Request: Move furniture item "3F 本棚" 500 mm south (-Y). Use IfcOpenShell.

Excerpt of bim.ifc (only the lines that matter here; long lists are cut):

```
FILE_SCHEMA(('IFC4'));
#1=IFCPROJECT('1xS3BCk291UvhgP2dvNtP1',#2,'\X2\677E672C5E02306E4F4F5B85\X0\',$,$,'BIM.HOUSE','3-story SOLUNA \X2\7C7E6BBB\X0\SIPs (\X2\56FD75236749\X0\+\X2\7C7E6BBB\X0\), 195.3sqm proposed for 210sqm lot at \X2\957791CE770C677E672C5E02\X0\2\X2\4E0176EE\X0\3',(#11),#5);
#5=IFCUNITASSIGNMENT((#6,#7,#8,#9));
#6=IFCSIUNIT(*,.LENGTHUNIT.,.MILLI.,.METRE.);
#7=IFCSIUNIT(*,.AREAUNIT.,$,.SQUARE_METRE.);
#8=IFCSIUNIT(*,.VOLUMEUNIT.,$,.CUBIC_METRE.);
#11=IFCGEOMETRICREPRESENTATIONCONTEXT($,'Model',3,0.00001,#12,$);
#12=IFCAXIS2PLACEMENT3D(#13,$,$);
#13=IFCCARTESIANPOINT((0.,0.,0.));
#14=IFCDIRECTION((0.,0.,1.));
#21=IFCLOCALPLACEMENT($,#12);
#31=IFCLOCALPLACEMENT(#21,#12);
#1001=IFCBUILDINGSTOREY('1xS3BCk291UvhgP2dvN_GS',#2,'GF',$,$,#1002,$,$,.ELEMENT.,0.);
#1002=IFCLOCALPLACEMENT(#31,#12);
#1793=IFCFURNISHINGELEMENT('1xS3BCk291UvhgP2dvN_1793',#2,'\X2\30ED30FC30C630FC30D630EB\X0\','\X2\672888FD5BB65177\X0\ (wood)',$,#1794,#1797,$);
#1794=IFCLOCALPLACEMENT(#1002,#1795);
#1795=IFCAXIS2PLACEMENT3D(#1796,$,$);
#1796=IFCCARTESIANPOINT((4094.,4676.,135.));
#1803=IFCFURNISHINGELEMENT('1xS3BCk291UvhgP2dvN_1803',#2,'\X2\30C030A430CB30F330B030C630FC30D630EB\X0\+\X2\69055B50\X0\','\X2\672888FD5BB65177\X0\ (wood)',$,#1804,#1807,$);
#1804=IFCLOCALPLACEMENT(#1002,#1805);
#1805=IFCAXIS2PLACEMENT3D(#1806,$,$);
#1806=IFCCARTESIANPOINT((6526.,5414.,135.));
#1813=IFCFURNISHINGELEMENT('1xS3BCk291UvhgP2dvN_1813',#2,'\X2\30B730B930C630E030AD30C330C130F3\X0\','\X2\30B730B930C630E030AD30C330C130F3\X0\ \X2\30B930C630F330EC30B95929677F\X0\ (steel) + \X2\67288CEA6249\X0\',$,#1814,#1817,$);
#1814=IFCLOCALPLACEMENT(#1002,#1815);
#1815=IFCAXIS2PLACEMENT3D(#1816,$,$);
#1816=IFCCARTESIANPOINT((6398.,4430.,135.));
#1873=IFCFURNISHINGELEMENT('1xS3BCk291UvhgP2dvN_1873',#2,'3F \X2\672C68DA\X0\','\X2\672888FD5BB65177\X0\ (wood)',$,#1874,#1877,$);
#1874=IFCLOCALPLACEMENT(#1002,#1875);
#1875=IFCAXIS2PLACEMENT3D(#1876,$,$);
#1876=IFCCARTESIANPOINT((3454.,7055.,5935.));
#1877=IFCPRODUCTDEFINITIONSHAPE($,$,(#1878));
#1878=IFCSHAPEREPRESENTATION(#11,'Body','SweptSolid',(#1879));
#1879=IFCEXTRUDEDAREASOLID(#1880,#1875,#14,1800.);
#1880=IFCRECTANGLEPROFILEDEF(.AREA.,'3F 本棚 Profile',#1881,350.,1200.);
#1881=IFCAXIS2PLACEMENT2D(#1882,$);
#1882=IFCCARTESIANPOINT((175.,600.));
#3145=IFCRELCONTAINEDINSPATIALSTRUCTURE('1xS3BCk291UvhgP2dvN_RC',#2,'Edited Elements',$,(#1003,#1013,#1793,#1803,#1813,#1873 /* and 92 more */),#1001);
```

```python
import ifcopenshell
import ifcopenshell.api.geometry
import ifcopenshell.util.placement
import ifcopenshell.util.unit

model = ifcopenshell.open("bim.ifc")
unit_scale = ifcopenshell.util.unit.calculate_unit_scale(model)

item = model.by_guid("1xS3BCk291UvhgP2dvN_1873")
matrix = ifcopenshell.util.placement.get_local_placement(item.ObjectPlacement)
matrix[1, 3] -= 0.5 / unit_scale
ifcopenshell.api.geometry.edit_object_placement(model, product=item, matrix=matrix, is_si=False)

print(ifcopenshell.util.placement.get_local_placement(item.ObjectPlacement).round(3) + 0.0)

model.write("bim_edited.ifc")
```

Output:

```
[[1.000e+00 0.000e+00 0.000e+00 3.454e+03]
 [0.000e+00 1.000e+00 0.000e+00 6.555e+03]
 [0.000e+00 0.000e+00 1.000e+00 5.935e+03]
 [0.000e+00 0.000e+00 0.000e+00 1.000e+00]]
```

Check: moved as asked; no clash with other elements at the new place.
